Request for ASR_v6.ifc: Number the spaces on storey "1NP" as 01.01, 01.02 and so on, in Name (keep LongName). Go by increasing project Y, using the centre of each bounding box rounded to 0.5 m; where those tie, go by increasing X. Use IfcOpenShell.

First a look at what the model holds.

```python
import ifcopenshell
import ifcopenshell.util.element
import ifcopenshell.util.placement

model = ifcopenshell.open("ASR_v6.ifc")
print(model.schema)
storey = next(s for s in model.by_type("IfcBuildingStorey") if s.Name == "1NP")
spaces = [e for e in ifcopenshell.util.element.get_decomposition(storey) if e.is_a("IfcSpace")]
for e in sorted(spaces, key=lambda e: e.id()):
    origin = ifcopenshell.util.placement.get_local_placement(e.ObjectPlacement)[:3, 3]
    print(e.id(), e.Name, e.LongName, origin.round(2) + 0.0, sep=" | ")
```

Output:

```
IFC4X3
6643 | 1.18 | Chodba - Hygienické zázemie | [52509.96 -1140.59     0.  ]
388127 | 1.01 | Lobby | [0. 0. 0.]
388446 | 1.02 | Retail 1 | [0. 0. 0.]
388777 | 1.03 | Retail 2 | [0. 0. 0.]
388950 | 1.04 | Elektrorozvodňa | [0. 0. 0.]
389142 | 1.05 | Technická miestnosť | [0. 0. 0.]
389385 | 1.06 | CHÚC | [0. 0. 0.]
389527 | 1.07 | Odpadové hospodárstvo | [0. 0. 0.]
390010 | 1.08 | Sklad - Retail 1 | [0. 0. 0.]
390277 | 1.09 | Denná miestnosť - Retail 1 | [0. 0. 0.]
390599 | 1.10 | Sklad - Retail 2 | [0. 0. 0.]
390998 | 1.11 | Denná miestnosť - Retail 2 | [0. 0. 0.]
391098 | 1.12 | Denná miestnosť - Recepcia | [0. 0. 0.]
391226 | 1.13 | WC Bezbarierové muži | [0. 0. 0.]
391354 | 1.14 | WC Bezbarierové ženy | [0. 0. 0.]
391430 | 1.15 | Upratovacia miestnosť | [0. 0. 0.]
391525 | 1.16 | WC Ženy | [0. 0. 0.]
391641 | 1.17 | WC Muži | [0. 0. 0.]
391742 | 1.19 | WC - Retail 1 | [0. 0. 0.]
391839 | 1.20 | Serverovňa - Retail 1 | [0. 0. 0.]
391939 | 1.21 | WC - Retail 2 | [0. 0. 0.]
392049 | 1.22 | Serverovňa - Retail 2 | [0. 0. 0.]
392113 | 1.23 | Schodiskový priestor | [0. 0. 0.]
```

```python
import ifcopenshell
import ifcopenshell.geom
import ifcopenshell.util.element
import ifcopenshell.util.shape

model = ifcopenshell.open("ASR_v6.ifc")
settings = ifcopenshell.geom.settings()
settings.set("use-world-coords", True)


def centre(element):
    shape = ifcopenshell.geom.create_shape(settings, element)
    return ifcopenshell.util.shape.get_bbox_centroid(shape.geometry)


storey = next(s for s in model.by_type("IfcBuildingStorey") if s.Name == "1NP")
spaces = [e for e in ifcopenshell.util.element.get_decomposition(storey) if e.is_a("IfcSpace")]

# Insertion points can sit at a corner or the storey origin, so sort by the geometry (in metres).
centres = {e: centre(e) for e in spaces}
spaces.sort(key=lambda e: (round(centres[e][1] / 0.5), centres[e][0]))

for i, e in enumerate(spaces, start=1):
    number = f"01.{i:02d}"
    e.Name = number
    print(e.id(), number)

model.write("ASR_v6_edited.ifc")
```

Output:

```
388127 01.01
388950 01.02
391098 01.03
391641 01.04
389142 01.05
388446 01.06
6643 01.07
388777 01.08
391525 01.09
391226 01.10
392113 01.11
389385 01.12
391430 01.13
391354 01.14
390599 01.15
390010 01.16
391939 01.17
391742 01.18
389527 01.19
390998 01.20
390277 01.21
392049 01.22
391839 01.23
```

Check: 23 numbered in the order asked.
